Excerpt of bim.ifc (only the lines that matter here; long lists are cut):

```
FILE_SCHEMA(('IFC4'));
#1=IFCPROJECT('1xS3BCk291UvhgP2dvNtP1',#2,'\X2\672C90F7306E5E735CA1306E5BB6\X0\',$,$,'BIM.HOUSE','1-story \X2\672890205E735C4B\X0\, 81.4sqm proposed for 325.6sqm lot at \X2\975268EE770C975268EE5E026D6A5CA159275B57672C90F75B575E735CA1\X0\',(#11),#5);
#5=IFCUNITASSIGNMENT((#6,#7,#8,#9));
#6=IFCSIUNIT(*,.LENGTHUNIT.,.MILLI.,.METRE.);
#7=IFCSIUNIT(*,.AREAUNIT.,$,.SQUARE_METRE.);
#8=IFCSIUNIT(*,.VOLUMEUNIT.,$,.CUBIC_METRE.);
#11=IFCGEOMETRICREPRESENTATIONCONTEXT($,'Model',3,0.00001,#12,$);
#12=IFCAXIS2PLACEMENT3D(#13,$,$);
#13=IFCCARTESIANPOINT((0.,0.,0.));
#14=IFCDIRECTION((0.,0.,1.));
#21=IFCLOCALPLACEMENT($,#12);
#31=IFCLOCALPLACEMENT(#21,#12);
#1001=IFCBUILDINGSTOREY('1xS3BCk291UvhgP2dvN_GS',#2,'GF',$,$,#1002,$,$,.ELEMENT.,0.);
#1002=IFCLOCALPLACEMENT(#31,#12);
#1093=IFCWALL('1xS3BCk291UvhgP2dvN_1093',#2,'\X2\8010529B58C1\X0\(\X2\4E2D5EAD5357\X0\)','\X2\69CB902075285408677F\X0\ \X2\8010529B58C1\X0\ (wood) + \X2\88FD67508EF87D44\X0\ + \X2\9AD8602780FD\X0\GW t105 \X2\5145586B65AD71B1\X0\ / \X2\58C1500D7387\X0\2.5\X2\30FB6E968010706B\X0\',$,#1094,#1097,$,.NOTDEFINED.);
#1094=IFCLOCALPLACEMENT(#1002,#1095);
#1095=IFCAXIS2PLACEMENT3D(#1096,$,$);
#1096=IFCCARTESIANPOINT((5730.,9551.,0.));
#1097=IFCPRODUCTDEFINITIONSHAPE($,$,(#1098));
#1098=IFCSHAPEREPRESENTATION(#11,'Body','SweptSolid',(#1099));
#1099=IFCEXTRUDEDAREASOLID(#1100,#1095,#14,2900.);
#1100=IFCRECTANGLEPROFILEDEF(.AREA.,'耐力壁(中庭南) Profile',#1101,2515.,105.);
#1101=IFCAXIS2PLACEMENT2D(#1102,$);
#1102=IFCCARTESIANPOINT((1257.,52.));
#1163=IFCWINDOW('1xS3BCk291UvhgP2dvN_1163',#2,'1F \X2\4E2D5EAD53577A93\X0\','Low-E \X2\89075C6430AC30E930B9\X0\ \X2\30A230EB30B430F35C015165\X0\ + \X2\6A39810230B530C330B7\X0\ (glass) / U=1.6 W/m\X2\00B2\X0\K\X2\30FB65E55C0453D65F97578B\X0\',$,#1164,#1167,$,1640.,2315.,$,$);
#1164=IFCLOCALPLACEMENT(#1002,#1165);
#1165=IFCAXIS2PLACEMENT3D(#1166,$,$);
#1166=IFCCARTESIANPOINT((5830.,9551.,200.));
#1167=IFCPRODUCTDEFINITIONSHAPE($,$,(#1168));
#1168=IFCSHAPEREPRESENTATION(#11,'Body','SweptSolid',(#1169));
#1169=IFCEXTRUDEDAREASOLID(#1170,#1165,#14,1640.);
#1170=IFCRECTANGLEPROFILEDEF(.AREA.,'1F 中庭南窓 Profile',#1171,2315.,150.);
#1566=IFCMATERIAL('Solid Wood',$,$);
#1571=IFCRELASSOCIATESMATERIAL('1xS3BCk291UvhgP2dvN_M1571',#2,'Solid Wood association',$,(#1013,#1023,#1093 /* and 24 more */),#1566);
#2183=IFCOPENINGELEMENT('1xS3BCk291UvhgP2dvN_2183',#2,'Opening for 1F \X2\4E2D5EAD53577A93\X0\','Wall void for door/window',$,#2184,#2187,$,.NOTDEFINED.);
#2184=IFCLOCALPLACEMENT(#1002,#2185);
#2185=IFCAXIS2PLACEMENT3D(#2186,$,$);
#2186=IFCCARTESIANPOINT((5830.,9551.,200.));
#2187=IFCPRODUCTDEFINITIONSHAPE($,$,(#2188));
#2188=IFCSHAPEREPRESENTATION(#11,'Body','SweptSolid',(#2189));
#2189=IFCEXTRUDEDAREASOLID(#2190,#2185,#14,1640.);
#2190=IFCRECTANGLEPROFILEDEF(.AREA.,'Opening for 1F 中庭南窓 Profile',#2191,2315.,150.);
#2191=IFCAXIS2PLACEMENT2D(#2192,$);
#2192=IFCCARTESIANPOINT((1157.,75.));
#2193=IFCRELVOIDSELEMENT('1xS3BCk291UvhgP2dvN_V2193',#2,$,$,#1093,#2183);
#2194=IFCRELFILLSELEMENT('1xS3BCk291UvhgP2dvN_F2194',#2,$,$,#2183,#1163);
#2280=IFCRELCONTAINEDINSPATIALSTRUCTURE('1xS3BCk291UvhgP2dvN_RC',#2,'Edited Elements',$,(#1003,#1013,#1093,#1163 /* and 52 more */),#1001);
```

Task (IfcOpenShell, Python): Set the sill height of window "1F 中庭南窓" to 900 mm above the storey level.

```python
import numpy as np
import ifcopenshell
import ifcopenshell.api.geometry
import ifcopenshell.geom
import ifcopenshell.util.element
import ifcopenshell.util.placement
import ifcopenshell.util.shape
import ifcopenshell.util.unit

model = ifcopenshell.open("bim.ifc")
unit_scale = ifcopenshell.util.unit.calculate_unit_scale(model)

window = model.by_guid("1xS3BCk291UvhgP2dvN_1163")
opening = window.FillsVoids[0].RelatingOpeningElement
storey = ifcopenshell.util.element.get_container(window, ifc_class="IfcBuildingStorey")
level = ifcopenshell.util.placement.get_local_placement(storey.ObjectPlacement)[2, 3]

# The opening's origin need not be at the sill, so measure its lowest point.
shape = ifcopenshell.geom.create_shape(ifcopenshell.geom.settings(), opening)
bottom = ifcopenshell.util.shape.get_shape_bottom_elevation(shape, shape.geometry) / unit_scale
dz = level + 900.0 - bottom

shift = np.array([0.0, 0.0, dz])
# The window is not placed relative to its opening, so move both.
for product in (opening, window):
    matrix = ifcopenshell.util.placement.get_local_placement(product.ObjectPlacement)
    matrix[:3, 3] += shift
    ifcopenshell.api.geometry.edit_object_placement(model, product=product, matrix=matrix, is_si=False)

print(f"moved by {dz * unit_scale:+.3f} m")

model.write("bim_updated.ifc")
```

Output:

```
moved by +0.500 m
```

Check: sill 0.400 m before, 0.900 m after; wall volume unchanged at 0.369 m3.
